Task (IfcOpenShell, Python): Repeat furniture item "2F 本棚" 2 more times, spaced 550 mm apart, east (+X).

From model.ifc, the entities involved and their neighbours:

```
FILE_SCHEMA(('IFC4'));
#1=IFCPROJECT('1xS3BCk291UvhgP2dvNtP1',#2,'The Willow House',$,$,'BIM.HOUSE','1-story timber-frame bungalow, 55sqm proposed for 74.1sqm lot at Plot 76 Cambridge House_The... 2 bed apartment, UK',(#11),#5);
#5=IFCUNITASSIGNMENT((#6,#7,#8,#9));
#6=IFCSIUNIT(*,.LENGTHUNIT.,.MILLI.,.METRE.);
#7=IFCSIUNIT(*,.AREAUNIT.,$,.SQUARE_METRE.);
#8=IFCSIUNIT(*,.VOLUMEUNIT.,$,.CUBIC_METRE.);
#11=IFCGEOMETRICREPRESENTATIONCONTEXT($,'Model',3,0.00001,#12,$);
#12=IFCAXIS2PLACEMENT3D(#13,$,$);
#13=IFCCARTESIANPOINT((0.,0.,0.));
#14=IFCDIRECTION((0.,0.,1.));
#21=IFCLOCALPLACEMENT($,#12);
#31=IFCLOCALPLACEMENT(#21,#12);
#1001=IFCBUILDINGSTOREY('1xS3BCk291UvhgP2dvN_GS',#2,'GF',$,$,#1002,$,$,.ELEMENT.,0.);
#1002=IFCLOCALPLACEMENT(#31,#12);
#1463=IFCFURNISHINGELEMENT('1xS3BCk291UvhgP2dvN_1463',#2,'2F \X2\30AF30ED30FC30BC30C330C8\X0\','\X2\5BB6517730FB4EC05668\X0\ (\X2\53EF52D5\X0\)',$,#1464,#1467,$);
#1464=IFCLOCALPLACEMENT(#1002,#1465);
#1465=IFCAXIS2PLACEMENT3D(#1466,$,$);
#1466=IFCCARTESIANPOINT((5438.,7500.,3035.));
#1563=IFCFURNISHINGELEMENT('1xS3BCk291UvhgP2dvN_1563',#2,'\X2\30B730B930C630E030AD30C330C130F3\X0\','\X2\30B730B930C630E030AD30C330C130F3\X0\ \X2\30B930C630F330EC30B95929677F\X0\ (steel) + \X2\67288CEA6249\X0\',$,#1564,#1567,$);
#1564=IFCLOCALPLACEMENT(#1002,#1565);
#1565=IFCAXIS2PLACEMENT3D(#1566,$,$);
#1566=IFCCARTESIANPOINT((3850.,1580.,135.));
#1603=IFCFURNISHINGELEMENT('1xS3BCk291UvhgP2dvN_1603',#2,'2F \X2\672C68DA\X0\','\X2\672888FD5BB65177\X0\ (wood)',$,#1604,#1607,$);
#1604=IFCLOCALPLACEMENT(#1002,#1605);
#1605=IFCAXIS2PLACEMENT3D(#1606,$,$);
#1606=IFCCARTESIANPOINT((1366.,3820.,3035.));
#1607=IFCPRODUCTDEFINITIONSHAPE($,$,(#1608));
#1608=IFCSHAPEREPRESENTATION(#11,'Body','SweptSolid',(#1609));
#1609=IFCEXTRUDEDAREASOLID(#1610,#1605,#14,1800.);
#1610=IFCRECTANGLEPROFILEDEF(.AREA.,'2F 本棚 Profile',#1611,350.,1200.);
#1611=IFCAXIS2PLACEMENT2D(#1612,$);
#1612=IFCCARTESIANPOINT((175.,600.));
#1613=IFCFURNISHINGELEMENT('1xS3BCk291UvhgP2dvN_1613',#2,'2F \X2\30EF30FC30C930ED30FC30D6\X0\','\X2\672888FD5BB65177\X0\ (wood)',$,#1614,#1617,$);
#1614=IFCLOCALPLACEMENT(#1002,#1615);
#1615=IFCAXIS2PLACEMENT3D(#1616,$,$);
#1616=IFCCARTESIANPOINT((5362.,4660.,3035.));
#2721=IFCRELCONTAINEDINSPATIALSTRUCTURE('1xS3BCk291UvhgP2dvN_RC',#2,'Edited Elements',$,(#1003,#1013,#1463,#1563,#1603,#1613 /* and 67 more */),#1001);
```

```python
import numpy as np
import ifcopenshell
import ifcopenshell.api.geometry
import ifcopenshell.api.root
import ifcopenshell.util.element
import ifcopenshell.util.placement
import ifcopenshell.util.unit

model = ifcopenshell.open("model.ifc")
unit_scale = ifcopenshell.util.unit.calculate_unit_scale(model)


def reuse_history(source, copy):
    """copy_class also copies each property set's owner history, people and application; keep the originals."""
    for rel in copy.IsDefinedBy:
        if rel.is_a("IfcRelDefinesByProperties") and (history := rel.RelatingPropertyDefinition.OwnerHistory):
            rel.RelatingPropertyDefinition.OwnerHistory = source.OwnerHistory
            ifcopenshell.util.element.remove_deep2(model, history)


source = model.by_guid("1xS3BCk291UvhgP2dvN_1603")
base = ifcopenshell.util.placement.get_local_placement(source.ObjectPlacement)
step = np.array([1.0, 0.0, 0.0]) * 0.55 / unit_scale

for i in range(1, 3):
    copy = ifcopenshell.api.root.copy_class(model, product=source)
    copy.Representation = ifcopenshell.util.element.copy_deep(
        model, source.Representation, exclude=["IfcGeometricRepresentationContext", "IfcRepresentationMap"]
    )
    reuse_history(source, copy)
    matrix = base.copy()
    matrix[:3, 3] += i * step
    print("added at", matrix[:3, 3].round(3) + 0.0)
    ifcopenshell.api.geometry.edit_object_placement(model, product=copy, matrix=matrix, is_si=False)

model.write("model_rev.ifc")
```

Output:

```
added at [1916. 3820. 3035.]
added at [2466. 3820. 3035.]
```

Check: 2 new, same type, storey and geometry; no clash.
